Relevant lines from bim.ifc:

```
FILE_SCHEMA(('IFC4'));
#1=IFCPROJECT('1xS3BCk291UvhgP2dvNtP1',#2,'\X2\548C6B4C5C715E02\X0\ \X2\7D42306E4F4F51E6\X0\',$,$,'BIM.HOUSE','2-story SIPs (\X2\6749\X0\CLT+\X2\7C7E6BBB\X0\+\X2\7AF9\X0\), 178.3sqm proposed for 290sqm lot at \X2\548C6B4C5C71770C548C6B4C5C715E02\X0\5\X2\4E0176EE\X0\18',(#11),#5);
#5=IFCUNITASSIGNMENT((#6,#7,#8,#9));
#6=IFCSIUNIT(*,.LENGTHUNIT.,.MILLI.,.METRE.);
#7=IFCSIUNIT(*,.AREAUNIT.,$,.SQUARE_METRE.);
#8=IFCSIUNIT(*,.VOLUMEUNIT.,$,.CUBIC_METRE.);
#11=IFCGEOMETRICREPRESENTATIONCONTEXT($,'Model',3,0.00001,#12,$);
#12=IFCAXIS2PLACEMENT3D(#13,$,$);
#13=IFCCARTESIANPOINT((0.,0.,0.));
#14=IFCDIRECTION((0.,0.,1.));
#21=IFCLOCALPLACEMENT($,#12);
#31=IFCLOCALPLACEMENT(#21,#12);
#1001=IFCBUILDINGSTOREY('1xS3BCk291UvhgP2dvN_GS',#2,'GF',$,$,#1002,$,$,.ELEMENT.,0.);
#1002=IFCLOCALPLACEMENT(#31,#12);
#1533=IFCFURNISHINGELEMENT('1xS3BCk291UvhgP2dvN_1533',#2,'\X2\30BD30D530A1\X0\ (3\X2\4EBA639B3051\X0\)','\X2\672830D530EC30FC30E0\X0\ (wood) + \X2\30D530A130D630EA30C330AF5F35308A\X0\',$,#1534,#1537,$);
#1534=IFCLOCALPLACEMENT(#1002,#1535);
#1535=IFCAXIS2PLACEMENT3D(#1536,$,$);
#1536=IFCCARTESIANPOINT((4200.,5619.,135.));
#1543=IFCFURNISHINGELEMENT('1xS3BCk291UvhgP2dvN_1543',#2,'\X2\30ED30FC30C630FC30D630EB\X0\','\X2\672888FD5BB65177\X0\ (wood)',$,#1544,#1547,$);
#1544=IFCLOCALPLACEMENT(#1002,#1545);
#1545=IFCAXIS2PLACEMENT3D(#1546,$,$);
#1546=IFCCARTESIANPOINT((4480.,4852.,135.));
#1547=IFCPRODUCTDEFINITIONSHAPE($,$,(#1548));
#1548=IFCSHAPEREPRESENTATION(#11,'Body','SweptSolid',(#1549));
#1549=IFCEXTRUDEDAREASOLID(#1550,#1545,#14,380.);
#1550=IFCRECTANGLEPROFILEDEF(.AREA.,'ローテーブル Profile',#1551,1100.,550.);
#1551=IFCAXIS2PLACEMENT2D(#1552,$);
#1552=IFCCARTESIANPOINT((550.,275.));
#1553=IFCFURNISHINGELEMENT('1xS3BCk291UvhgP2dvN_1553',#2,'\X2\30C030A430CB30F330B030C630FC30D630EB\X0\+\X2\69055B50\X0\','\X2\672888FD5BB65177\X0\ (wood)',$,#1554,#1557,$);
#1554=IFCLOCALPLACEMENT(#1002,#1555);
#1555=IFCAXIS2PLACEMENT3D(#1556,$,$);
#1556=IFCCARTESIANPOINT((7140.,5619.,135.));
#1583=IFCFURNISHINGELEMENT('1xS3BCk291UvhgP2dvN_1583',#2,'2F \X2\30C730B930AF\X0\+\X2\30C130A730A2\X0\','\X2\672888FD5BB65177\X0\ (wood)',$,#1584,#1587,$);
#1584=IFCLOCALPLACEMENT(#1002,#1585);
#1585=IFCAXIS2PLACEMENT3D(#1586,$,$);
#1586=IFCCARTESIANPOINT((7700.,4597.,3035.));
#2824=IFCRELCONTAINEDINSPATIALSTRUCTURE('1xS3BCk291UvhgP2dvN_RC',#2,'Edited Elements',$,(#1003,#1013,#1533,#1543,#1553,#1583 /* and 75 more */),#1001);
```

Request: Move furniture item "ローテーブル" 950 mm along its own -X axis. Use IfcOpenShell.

```python
import ifcopenshell
import ifcopenshell.api.geometry
import ifcopenshell.util.placement
import ifcopenshell.util.unit

model = ifcopenshell.open("bim.ifc")
unit_scale = ifcopenshell.util.unit.calculate_unit_scale(model)

item = model.by_guid("1xS3BCk291UvhgP2dvN_1543")
matrix = ifcopenshell.util.placement.get_local_placement(item.ObjectPlacement)
matrix[:3, 3] -= matrix[:3, 0] * 0.95 / unit_scale
ifcopenshell.api.geometry.edit_object_placement(model, product=item, matrix=matrix, is_si=False)

print(ifcopenshell.util.placement.get_local_placement(item.ObjectPlacement).round(3) + 0.0)

model.write("bim_rev.ifc")
```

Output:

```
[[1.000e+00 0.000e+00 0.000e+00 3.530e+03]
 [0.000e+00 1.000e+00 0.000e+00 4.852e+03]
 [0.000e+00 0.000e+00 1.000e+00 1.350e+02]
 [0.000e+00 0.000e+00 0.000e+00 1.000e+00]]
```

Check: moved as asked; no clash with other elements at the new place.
